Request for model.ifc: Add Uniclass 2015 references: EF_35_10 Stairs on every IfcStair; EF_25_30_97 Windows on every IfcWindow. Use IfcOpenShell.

First a look at what the model holds.

```python
import ifcopenshell

model = ifcopenshell.open("model.ifc")
print(model.schema)
print("classifications:", [c.Name for c in model.by_type("IfcClassification")])
for ifc_class in ("IfcDoor", "IfcRoof", "IfcStair", "IfcWall", "IfcWindow"):
    print(ifc_class, len(model.by_type(ifc_class)))
```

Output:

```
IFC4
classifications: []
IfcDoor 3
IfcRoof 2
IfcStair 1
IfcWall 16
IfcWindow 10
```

```python
import ifcopenshell
import ifcopenshell.api.classification

model = ifcopenshell.open("model.ifc")

system = ifcopenshell.api.classification.add_classification(model, classification="Uniclass 2015")

codes = {
    "IfcStair": ("EF_35_10", "Stairs"),
    "IfcWindow": ("EF_25_30_97", "Windows"),
}
for ifc_class, (code, name) in codes.items():
    products = model.by_type(ifc_class)
    ifcopenshell.api.classification.add_reference(
        model, products=products, classification=system, identification=code, name=name
    )
    print(code, len(products))

model.write("model_rev.ifc")
```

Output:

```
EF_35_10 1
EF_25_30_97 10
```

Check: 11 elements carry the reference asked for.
